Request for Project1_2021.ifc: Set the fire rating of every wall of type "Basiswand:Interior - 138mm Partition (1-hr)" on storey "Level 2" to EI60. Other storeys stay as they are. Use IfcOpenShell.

First a look at what the model holds.

```python
import ifcopenshell
import ifcopenshell.util.element

model = ifcopenshell.open("Project1_2021.ifc")
print(model.schema)
storey = next(s for s in model.by_type("IfcBuildingStorey") if s.Name == "Level 2")
walls = [e for e in ifcopenshell.util.element.get_decomposition(storey) if e.is_a("IfcWall")]
seen = {}
for e in walls:
    element_type = ifcopenshell.util.element.get_type(e)
    key = (element_type.Name if element_type != e and element_type else None, ifcopenshell.util.element.get_pset(e, "Pset_WallCommon", "FireRating"))
    seen[key] = seen.get(key, 0) + 1
for (name, value), count in sorted(seen.items(), key=str):
    print(count, "x", name, "|", value)
```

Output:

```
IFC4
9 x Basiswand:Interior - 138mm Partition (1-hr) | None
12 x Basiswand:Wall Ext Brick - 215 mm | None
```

```python
import ifcopenshell
import ifcopenshell.api.pset
import ifcopenshell.util.element

model = ifcopenshell.open("Project1_2021.ifc")

storey = next(s for s in model.by_type("IfcBuildingStorey") if s.Name == "Level 2")
walls = [e for e in ifcopenshell.util.element.get_decomposition(storey) if e.is_a("IfcWall")]

count = 0
for e in walls:
    element_type = ifcopenshell.util.element.get_type(e)
    if element_type in (None, e) or element_type.Name != "Basiswand:Interior - 138mm Partition (1-hr)":
        continue
    # add_pset returns the element's existing set when there is one.
    pset = ifcopenshell.api.pset.add_pset(model, product=e, name="Pset_WallCommon")
    ifcopenshell.api.pset.edit_pset(model, pset=pset, properties={"FireRating": "EI60"})
    count += 1

print(count, "walls updated")

model.write("Project1_2021_edited.ifc")
```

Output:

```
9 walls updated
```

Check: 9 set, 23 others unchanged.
